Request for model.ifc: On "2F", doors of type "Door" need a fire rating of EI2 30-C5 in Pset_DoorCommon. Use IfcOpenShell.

First a look at what the model holds.

```python
import ifcopenshell
import ifcopenshell.util.element

model = ifcopenshell.open("model.ifc")
print(model.schema)
storey = next(s for s in model.by_type("IfcBuildingStorey") if s.Name == "2F")
doors = [e for e in ifcopenshell.util.element.get_decomposition(storey) if e.is_a("IfcDoor")]
seen = {}
for e in doors:
    element_type = ifcopenshell.util.element.get_type(e)
    key = (element_type.Name if element_type != e and element_type else None, ifcopenshell.util.element.get_pset(e, "Pset_DoorCommon", "FireRating"))
    seen[key] = seen.get(key, 0) + 1
for (name, value), count in sorted(seen.items(), key=str):
    print(count, "x", name, "|", value)
```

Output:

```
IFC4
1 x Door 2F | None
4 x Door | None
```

```python
import ifcopenshell
import ifcopenshell.api.pset
import ifcopenshell.util.element

model = ifcopenshell.open("model.ifc")

storey = next(s for s in model.by_type("IfcBuildingStorey") if s.Name == "2F")
doors = [e for e in ifcopenshell.util.element.get_decomposition(storey) if e.is_a("IfcDoor")]

count = 0
for e in doors:
    element_type = ifcopenshell.util.element.get_type(e)
    if element_type in (None, e) or element_type.Name != "Door":
        continue
    # add_pset returns the element's existing set when there is one.
    pset = ifcopenshell.api.pset.add_pset(model, product=e, name="Pset_DoorCommon")
    ifcopenshell.api.pset.edit_pset(model, pset=pset, properties={"FireRating": "EI2 30-C5"})
    count += 1

print(count, "doors updated")

model.write("model_updated.ifc")
```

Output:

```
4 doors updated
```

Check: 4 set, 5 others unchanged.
